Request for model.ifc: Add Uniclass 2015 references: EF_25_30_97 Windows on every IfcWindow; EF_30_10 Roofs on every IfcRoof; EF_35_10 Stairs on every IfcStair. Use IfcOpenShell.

First a look at what the model holds.

```python
import ifcopenshell

model = ifcopenshell.open("model.ifc")
print(model.schema)
print("classifications:", [c.Name for c in model.by_type("IfcClassification")])
for ifc_class in ("IfcDoor", "IfcRoof", "IfcStair", "IfcWall", "IfcWindow"):
    print(ifc_class, len(model.by_type(ifc_class)))
```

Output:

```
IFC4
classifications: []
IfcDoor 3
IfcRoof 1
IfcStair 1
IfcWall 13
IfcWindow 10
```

```python
import ifcopenshell
import ifcopenshell.api.classification

model = ifcopenshell.open("model.ifc")

system = ifcopenshell.api.classification.add_classification(model, classification="Uniclass 2015")

codes = {
    "IfcWindow": ("EF_25_30_97", "Windows"),
    "IfcRoof": ("EF_30_10", "Roofs"),
    "IfcStair": ("EF_35_10", "Stairs"),
}
for ifc_class, (code, name) in codes.items():
    products = model.by_type(ifc_class)
    ifcopenshell.api.classification.add_reference(
        model, products=products, classification=system, identification=code, name=name
    )
    print(code, len(products))

model.write("model_edited.ifc")
```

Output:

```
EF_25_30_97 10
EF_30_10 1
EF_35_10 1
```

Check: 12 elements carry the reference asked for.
